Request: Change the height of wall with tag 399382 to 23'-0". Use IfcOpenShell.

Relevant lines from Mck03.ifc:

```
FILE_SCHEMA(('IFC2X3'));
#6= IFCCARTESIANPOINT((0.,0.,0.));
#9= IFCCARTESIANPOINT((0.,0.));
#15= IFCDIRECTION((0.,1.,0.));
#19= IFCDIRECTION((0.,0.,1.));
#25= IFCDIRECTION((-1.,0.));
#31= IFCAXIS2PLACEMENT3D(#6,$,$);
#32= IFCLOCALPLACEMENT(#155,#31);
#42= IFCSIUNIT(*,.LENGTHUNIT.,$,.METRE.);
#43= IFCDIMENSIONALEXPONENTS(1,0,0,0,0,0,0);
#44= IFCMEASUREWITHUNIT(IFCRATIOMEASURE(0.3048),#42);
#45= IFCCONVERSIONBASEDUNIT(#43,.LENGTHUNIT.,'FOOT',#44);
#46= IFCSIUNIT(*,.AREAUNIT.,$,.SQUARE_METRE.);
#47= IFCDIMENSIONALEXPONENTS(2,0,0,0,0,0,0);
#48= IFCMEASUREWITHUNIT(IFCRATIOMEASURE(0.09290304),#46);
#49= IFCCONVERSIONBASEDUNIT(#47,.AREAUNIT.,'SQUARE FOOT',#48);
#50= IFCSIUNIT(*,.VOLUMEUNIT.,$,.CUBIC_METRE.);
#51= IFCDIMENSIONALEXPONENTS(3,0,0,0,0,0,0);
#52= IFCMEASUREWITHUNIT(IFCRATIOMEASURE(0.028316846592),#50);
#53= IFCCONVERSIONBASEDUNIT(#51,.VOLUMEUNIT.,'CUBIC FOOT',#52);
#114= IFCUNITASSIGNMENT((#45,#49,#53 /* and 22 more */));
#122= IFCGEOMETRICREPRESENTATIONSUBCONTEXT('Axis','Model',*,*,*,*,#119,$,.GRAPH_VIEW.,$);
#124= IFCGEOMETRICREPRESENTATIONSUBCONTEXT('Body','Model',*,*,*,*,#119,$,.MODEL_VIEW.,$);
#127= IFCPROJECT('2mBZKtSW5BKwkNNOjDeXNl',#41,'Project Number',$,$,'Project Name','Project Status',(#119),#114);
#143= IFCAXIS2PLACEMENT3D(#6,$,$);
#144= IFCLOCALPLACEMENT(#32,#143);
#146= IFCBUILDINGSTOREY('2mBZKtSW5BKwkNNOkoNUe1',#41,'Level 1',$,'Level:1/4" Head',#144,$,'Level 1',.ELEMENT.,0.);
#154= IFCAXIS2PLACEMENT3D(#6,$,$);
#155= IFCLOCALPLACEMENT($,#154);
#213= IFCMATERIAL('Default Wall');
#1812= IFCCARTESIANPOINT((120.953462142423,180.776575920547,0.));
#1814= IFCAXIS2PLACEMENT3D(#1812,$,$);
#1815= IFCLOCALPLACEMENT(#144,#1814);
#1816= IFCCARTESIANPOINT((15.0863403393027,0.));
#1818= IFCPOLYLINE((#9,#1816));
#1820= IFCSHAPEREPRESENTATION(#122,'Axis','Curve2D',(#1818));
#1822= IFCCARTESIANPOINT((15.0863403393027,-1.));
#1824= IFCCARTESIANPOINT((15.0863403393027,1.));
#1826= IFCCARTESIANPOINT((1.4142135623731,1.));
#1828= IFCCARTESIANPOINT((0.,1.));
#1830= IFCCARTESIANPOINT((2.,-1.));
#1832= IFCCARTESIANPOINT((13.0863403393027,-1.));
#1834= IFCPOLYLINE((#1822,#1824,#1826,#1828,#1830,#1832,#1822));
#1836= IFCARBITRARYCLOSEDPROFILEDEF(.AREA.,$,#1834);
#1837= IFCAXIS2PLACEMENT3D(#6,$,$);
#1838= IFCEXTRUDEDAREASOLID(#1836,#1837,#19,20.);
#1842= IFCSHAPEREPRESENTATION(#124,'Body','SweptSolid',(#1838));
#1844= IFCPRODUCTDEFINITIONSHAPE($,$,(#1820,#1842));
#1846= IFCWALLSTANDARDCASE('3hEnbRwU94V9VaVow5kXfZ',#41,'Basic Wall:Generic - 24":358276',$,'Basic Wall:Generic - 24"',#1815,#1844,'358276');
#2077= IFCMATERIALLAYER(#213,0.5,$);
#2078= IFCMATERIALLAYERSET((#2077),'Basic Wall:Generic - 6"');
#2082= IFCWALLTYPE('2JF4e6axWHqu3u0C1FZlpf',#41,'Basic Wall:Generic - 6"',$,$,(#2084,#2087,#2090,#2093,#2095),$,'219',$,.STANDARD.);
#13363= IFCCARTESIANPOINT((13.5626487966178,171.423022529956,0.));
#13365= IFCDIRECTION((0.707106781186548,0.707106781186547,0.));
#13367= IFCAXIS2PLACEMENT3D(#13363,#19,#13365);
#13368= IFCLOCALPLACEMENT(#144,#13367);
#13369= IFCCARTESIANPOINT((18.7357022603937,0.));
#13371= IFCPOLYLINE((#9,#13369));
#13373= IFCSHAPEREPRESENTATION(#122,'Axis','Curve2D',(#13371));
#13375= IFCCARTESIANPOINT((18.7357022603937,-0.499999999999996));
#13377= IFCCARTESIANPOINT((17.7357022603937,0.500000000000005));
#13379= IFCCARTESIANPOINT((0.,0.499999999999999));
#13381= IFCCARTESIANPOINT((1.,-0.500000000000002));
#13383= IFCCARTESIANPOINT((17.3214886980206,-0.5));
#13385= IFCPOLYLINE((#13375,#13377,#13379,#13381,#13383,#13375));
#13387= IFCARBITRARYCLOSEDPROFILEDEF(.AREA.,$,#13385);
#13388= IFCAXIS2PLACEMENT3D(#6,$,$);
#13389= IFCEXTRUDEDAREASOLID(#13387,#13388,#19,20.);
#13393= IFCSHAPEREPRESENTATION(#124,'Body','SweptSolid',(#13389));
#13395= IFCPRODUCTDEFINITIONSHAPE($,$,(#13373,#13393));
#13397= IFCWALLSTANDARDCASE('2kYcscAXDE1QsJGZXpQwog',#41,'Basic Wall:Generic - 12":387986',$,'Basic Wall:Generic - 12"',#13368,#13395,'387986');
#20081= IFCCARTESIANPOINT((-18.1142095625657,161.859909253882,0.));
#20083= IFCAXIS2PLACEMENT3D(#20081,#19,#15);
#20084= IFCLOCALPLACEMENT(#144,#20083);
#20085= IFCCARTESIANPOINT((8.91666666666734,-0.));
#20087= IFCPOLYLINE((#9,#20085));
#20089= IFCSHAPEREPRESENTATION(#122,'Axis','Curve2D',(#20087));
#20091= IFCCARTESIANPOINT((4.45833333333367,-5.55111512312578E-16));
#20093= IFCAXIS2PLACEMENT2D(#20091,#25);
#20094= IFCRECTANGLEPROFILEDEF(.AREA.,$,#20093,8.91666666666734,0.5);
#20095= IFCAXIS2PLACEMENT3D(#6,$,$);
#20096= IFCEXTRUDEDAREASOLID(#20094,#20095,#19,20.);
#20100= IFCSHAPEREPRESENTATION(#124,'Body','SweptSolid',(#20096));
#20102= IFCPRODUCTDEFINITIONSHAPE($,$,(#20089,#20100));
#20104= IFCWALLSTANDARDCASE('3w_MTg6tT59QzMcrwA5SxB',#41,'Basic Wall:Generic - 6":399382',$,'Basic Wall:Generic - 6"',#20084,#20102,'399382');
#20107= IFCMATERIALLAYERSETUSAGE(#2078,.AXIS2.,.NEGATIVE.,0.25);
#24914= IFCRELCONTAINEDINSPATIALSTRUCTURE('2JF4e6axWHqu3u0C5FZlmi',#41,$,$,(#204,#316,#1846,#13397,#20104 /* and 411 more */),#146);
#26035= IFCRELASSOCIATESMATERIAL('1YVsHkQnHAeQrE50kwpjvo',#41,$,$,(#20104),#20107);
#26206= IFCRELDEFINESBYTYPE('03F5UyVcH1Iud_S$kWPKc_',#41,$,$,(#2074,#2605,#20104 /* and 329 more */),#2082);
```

```python
import ifcopenshell
import ifcopenshell.geom
import ifcopenshell.util.representation
import ifcopenshell.util.shape
import ifcopenshell.util.unit

model = ifcopenshell.open("Mck03.ifc")
unit_scale = ifcopenshell.util.unit.calculate_unit_scale(model)
settings = ifcopenshell.geom.settings()


def volume(element):
    """Net volume in cubic metres, openings subtracted."""
    shape = ifcopenshell.geom.create_shape(settings, element)
    return ifcopenshell.util.shape.get_volume(shape.geometry)


wall = model.by_guid("3w_MTg6tT59QzMcrwA5SxB")
before = volume(wall)

body = ifcopenshell.util.representation.get_representation(wall, "Model", "Body")
solid = body.Items[0]
old_height = solid.Depth
solid.Depth = 276 * 0.0254 / unit_scale
after = volume(wall)

print(f"height {old_height:g} -> {solid.Depth:g}, volume {before:.3f} -> {after:.3f} m3")

model.write("Mck03-out.ifc")
```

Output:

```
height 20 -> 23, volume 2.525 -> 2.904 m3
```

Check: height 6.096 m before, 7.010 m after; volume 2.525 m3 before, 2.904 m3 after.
